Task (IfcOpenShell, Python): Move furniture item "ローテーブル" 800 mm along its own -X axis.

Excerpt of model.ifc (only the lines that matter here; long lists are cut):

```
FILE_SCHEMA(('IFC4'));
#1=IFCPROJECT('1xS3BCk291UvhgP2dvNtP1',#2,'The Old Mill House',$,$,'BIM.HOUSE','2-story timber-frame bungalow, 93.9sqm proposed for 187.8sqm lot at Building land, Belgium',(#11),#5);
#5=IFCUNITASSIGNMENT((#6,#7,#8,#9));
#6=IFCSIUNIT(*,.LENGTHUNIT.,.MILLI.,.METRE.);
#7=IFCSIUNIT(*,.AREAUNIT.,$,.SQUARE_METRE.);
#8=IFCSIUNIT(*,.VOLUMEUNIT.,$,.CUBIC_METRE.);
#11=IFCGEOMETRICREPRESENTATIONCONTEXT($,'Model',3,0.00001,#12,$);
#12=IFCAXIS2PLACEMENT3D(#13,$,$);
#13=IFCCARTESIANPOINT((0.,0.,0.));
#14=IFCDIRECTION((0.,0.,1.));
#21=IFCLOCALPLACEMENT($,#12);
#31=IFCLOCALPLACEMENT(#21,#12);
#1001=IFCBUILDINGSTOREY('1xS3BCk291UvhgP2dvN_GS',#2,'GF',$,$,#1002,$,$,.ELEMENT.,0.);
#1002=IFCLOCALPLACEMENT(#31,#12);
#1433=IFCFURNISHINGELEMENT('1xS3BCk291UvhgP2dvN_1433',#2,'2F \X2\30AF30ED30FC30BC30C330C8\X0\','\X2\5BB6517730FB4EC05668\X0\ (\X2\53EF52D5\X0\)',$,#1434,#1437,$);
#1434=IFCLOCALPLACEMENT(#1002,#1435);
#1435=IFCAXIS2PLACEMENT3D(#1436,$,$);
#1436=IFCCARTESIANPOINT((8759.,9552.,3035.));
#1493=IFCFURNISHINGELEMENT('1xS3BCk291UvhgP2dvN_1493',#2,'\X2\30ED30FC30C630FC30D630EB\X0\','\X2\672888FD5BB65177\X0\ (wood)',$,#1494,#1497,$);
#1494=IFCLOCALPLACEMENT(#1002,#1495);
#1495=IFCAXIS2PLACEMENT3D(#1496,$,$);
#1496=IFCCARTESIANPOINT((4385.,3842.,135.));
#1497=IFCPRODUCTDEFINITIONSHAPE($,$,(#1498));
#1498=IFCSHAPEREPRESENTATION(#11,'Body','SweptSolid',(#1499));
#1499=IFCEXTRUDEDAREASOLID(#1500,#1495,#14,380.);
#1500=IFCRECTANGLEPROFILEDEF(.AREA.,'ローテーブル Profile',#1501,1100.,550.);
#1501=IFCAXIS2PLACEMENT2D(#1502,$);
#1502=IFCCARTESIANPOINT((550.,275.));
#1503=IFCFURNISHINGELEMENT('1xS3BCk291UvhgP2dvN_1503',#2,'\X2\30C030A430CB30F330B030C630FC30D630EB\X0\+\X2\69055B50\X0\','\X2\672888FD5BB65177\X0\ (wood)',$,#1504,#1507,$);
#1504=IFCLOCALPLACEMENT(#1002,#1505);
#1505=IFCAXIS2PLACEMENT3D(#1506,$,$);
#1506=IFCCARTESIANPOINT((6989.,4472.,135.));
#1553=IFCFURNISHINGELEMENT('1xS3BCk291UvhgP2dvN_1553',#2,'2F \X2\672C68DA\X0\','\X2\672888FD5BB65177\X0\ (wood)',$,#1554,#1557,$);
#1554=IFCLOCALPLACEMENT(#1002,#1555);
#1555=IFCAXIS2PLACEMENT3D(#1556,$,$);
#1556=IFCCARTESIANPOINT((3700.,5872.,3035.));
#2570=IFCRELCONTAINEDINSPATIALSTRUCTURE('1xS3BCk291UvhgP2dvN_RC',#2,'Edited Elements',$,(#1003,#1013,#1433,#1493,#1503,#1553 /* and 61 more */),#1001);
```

```python
import ifcopenshell
import ifcopenshell.api.geometry
import ifcopenshell.util.placement

model = ifcopenshell.open("model.ifc")

item = model.by_id(1493)
matrix = ifcopenshell.util.placement.get_local_placement(item.ObjectPlacement)
matrix[:3, 3] -= matrix[:3, 0] * 800.0
ifcopenshell.api.geometry.edit_object_placement(model, product=item, matrix=matrix, is_si=False)

print(ifcopenshell.util.placement.get_local_placement(item.ObjectPlacement).round(3) + 0.0)

model.write("model_rev.ifc")
```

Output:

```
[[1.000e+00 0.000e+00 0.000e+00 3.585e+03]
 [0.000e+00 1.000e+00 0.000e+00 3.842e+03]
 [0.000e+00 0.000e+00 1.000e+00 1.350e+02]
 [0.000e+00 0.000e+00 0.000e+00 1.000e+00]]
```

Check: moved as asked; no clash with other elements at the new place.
